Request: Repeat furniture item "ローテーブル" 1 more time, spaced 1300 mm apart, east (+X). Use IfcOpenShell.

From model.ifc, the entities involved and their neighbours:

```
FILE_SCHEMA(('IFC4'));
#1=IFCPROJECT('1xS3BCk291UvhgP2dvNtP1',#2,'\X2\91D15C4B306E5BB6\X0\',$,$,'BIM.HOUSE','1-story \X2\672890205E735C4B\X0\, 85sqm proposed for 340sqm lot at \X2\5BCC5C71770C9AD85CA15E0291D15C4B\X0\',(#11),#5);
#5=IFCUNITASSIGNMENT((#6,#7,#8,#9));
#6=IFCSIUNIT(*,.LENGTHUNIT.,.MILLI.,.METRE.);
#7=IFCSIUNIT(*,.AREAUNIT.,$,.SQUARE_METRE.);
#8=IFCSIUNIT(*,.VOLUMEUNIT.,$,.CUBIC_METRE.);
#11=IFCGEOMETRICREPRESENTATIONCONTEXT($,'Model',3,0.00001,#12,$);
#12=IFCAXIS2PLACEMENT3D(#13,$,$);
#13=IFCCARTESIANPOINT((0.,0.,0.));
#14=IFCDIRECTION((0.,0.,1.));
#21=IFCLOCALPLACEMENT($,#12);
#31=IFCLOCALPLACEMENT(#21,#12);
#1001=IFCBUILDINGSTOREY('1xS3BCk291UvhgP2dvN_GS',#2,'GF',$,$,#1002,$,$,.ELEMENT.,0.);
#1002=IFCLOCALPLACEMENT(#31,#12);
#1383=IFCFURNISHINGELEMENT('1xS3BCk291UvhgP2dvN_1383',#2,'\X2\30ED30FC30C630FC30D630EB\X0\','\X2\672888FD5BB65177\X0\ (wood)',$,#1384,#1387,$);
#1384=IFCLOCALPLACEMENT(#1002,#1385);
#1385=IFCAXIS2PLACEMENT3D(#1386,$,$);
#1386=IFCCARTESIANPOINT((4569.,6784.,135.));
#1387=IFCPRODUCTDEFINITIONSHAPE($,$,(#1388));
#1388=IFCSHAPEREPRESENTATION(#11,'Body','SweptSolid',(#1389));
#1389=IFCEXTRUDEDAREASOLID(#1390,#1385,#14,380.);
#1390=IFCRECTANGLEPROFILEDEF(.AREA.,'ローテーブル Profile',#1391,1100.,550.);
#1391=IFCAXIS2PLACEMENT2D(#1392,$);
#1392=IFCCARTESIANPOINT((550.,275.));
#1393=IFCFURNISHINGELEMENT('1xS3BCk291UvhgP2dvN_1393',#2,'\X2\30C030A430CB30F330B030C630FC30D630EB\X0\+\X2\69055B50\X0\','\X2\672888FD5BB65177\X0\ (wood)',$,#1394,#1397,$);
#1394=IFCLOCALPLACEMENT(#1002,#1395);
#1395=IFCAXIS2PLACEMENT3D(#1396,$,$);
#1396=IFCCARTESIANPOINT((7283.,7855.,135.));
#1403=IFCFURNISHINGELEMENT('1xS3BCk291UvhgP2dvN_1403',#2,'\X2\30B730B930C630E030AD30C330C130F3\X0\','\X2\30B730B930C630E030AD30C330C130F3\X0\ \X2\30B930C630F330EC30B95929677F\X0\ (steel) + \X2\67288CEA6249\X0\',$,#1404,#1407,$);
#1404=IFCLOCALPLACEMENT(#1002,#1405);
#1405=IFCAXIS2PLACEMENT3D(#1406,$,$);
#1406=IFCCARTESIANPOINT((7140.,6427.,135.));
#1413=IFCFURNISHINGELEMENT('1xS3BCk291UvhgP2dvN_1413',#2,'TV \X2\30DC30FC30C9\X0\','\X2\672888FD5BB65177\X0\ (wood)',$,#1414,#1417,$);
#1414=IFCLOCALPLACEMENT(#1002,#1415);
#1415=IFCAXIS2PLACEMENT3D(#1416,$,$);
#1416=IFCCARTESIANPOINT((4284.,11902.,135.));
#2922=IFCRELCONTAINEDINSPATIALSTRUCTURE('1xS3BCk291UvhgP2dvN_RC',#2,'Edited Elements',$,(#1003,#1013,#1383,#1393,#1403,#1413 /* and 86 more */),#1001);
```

```python
import numpy as np
import ifcopenshell
import ifcopenshell.api.geometry
import ifcopenshell.api.root
import ifcopenshell.util.element
import ifcopenshell.util.placement

model = ifcopenshell.open("model.ifc")


def reuse_history(source, copy):
    """copy_class also copies each property set's owner history, people and application; keep the originals."""
    for rel in copy.IsDefinedBy:
        if rel.is_a("IfcRelDefinesByProperties") and (history := rel.RelatingPropertyDefinition.OwnerHistory):
            rel.RelatingPropertyDefinition.OwnerHistory = source.OwnerHistory
            ifcopenshell.util.element.remove_deep2(model, history)


source = model.by_guid("1xS3BCk291UvhgP2dvN_1383")
base = ifcopenshell.util.placement.get_local_placement(source.ObjectPlacement)
step = np.array([1.0, 0.0, 0.0]) * 1300.0

for i in range(1, 2):
    copy = ifcopenshell.api.root.copy_class(model, product=source)
    copy.Representation = ifcopenshell.util.element.copy_deep(
        model, source.Representation, exclude=["IfcGeometricRepresentationContext", "IfcRepresentationMap"]
    )
    reuse_history(source, copy)
    matrix = base.copy()
    matrix[:3, 3] += i * step
    print("added at", matrix[:3, 3].round(3) + 0.0)
    ifcopenshell.api.geometry.edit_object_placement(model, product=copy, matrix=matrix, is_si=False)

model.write("model_updated.ifc")
```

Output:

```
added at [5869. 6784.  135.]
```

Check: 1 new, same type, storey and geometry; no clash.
